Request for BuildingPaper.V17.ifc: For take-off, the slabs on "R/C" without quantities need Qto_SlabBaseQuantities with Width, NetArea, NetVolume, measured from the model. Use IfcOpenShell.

First a look at what the model holds.

```python
import ifcopenshell
import ifcopenshell.util.element
import ifcopenshell.util.unit

model = ifcopenshell.open("BuildingPaper.V17.ifc")
print(model.schema)
for unit_type in ("LENGTHUNIT", "AREAUNIT", "VOLUMEUNIT"):
    print(unit_type, ifcopenshell.util.unit.calculate_unit_scale(model, unit_type))
storey = next(s for s in model.by_type("IfcBuildingStorey") if s.Name == "R/C")
slabs = [e for e in ifcopenshell.util.element.get_decomposition(storey) if e.is_a("IfcSlab")]
for e in sorted(slabs, key=lambda e: e.id()):
    print(e.id(), e.is_a(), e.Name, list(ifcopenshell.util.element.get_psets(e, qtos_only=True)), sep=" | ")
```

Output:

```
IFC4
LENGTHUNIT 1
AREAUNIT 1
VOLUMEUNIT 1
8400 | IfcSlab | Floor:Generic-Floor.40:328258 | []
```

```python
import ifcopenshell
import ifcopenshell.api.pset
import ifcopenshell.geom
import ifcopenshell.util.element
import ifcopenshell.util.shape
import ifcopenshell.util.unit

model = ifcopenshell.open("BuildingPaper.V17.ifc")
unit_scale = ifcopenshell.util.unit.calculate_unit_scale(model)
area_scale = ifcopenshell.util.unit.calculate_unit_scale(model, "AREAUNIT")
volume_scale = ifcopenshell.util.unit.calculate_unit_scale(model, "VOLUMEUNIT")
settings = ifcopenshell.geom.settings()

storey = next(s for s in model.by_type("IfcBuildingStorey") if s.Name == "R/C")
slabs = [e for e in ifcopenshell.util.element.get_decomposition(storey) if e.is_a("IfcSlab")]

for e in sorted(slabs, key=lambda e: e.id()):
    if ifcopenshell.util.element.get_psets(e, qtos_only=True, should_inherit=False):
        continue
    # Geometry comes back in metres, in the element's own axes.
    shape = ifcopenshell.geom.create_shape(settings, e)
    values = {
        "Width": ifcopenshell.util.shape.get_z(shape.geometry) / unit_scale,
        "NetArea": ifcopenshell.util.shape.get_footprint_area(shape.geometry) / area_scale,
        "NetVolume": ifcopenshell.util.shape.get_volume(shape.geometry) / volume_scale,
    }
    qto = ifcopenshell.api.pset.add_qto(model, product=e, name="Qto_SlabBaseQuantities")
    ifcopenshell.api.pset.edit_qto(model, qto=qto, properties=values)
    print(e.id(), {k: round(v, 3) for k, v in values.items()})

model.write("BuildingPaper.V17_updated.ifc")
```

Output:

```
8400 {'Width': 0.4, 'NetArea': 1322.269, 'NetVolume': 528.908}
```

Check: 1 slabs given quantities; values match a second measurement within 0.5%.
